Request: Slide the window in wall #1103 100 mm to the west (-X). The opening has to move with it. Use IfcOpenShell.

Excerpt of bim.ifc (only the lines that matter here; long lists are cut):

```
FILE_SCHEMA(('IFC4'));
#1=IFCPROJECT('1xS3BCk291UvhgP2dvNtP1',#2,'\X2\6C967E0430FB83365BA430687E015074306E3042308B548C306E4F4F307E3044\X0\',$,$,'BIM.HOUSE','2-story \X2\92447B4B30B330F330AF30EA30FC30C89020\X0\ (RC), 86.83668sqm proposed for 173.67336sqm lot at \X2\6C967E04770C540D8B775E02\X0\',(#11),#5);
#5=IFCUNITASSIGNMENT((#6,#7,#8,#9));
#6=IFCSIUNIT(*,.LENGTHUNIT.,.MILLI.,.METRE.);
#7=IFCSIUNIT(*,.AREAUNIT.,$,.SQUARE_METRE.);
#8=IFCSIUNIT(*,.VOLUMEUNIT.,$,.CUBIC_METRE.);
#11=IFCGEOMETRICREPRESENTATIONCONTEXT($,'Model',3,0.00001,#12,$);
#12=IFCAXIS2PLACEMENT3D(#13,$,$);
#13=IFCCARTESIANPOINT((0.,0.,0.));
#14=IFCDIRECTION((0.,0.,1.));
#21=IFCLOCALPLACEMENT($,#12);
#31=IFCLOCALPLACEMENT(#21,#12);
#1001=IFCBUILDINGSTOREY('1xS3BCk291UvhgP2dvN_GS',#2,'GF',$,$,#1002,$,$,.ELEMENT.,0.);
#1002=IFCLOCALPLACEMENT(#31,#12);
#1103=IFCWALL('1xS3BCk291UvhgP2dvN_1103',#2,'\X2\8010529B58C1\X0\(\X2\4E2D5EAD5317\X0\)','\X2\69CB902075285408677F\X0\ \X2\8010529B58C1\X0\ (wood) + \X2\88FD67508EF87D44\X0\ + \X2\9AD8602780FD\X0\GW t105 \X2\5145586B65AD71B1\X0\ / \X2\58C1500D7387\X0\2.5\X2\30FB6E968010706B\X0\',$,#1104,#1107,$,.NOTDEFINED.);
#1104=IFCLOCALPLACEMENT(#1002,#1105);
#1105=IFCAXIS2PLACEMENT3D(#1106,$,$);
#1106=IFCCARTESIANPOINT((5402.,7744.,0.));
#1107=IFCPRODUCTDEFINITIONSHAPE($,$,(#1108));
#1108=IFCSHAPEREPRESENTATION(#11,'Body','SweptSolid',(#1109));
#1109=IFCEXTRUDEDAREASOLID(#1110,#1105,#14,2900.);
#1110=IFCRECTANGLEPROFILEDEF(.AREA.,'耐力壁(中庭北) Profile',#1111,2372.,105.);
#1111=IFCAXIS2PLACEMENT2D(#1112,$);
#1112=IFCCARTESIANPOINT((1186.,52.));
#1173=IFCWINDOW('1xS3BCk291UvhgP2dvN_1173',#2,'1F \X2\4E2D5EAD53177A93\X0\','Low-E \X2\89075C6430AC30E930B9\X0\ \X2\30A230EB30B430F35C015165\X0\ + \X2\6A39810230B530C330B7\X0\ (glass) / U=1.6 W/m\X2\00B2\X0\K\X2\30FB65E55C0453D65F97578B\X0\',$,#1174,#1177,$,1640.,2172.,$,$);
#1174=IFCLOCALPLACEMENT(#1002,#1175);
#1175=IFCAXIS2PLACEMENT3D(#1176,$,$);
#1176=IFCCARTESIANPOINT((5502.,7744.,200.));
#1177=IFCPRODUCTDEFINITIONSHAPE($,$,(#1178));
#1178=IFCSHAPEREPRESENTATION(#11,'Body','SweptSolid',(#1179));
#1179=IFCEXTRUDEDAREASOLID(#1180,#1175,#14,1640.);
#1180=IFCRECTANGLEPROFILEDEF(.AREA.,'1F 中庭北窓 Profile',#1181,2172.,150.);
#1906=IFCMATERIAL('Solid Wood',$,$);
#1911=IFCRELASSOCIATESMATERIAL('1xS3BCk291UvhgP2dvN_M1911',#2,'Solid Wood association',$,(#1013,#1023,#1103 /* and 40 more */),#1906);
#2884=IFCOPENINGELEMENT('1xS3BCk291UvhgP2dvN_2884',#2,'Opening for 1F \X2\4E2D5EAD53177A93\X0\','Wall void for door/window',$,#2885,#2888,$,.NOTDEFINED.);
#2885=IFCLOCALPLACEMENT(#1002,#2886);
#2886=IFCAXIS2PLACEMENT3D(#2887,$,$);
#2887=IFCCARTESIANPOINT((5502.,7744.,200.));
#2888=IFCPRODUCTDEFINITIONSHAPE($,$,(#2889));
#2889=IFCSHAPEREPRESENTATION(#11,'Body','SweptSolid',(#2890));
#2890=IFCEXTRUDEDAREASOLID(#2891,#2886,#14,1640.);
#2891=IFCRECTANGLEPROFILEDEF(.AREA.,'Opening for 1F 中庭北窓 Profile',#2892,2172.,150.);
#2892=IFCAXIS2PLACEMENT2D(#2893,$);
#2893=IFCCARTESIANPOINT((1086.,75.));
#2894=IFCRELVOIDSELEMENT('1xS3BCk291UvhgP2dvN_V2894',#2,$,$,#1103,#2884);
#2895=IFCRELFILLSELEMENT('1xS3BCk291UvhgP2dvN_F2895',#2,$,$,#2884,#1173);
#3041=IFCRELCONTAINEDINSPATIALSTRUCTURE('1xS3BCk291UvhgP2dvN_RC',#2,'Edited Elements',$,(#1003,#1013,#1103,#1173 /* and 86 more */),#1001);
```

```python
import ifcopenshell
import ifcopenshell.api.geometry
import ifcopenshell.util.placement
import ifcopenshell.util.unit

model = ifcopenshell.open("bim.ifc")
unit_scale = ifcopenshell.util.unit.calculate_unit_scale(model)

window = model.by_guid("1xS3BCk291UvhgP2dvN_1173")
opening = window.FillsVoids[0].RelatingOpeningElement
wall = opening.VoidsElements[0].RelatingBuildingElement

wall_matrix = ifcopenshell.util.placement.get_local_placement(wall.ObjectPlacement)
shift = wall_matrix[:3, 0] * -0.1 / unit_scale
before = ifcopenshell.util.placement.get_local_placement(window.ObjectPlacement)[:3, 3].copy()

# The window is not placed relative to its opening, so move both.
for product in (opening, window):
    matrix = ifcopenshell.util.placement.get_local_placement(product.ObjectPlacement)
    matrix[:3, 3] += shift
    ifcopenshell.api.geometry.edit_object_placement(model, product=product, matrix=matrix, is_si=False)

after = ifcopenshell.util.placement.get_local_placement(window.ObjectPlacement)[:3, 3]
print("window moved by", (after - before).round(3) + 0.0)

model.write("bim_updated.ifc")
```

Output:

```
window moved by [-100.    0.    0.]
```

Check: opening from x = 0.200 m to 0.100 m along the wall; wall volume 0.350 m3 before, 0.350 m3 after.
